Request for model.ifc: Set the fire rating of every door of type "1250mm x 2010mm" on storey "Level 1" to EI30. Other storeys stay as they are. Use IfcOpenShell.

First a look at what the model holds.

```python
import ifcopenshell
import ifcopenshell.util.element

model = ifcopenshell.open("model.ifc")
print(model.schema)
storey = next(s for s in model.by_type("IfcBuildingStorey") if s.Name == "Level 1")
doors = [e for e in ifcopenshell.util.element.get_decomposition(storey) if e.is_a("IfcDoor")]
seen = {}
for e in doors:
    element_type = ifcopenshell.util.element.get_type(e)
    key = (element_type.Name if element_type != e and element_type else None, ifcopenshell.util.element.get_pset(e, "Pset_DoorCommon", "FireRating"))
    seen[key] = seen.get(key, 0) + 1
for (name, value), count in sorted(seen.items(), key=str):
    print(count, "x", name, "|", value)
```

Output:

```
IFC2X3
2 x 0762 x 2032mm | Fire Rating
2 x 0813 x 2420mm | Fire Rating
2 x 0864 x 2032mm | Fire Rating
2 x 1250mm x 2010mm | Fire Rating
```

```python
import ifcopenshell
import ifcopenshell.api.pset
import ifcopenshell.util.element

model = ifcopenshell.open("model.ifc")

storey = next(s for s in model.by_type("IfcBuildingStorey") if s.Name == "Level 1")
doors = [e for e in ifcopenshell.util.element.get_decomposition(storey) if e.is_a("IfcDoor")]

count = 0
for e in doors:
    element_type = ifcopenshell.util.element.get_type(e)
    if element_type in (None, e) or element_type.Name != "1250mm x 2010mm":
        continue
    # add_pset returns the element's existing set when there is one.
    pset = ifcopenshell.api.pset.add_pset(model, product=e, name="Pset_DoorCommon")
    ifcopenshell.api.pset.edit_pset(model, pset=pset, properties={"FireRating": "EI30"})
    count += 1

print(count, "doors updated")

model.write("model-out.ifc")
```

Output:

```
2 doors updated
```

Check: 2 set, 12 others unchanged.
